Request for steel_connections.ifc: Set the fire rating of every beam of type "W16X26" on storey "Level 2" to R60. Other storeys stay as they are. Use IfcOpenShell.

First a look at what the model holds.

```python
import ifcopenshell
import ifcopenshell.util.element

model = ifcopenshell.open("steel_connections.ifc")
print(model.schema)
storey = next(s for s in model.by_type("IfcBuildingStorey") if s.Name == "Level 2")
beams = [e for e in ifcopenshell.util.element.get_decomposition(storey) if e.is_a("IfcBeam")]
seen = {}
for e in beams:
    element_type = ifcopenshell.util.element.get_type(e)
    key = (element_type.Name if element_type != e and element_type else None, ifcopenshell.util.element.get_pset(e, "Pset_BeamCommon", "FireRating"))
    seen[key] = seen.get(key, 0) + 1
for (name, value), count in sorted(seen.items(), key=str):
    print(count, "x", name, "|", value)
```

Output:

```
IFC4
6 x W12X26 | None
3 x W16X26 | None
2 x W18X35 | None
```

```python
import ifcopenshell
import ifcopenshell.api.pset
import ifcopenshell.util.element

model = ifcopenshell.open("steel_connections.ifc")

storey = next(s for s in model.by_type("IfcBuildingStorey") if s.Name == "Level 2")
beams = [e for e in ifcopenshell.util.element.get_decomposition(storey) if e.is_a("IfcBeam")]

count = 0
for e in beams:
    element_type = ifcopenshell.util.element.get_type(e)
    if element_type in (None, e) or element_type.Name != "W16X26":
        continue
    # add_pset returns the element's existing set when there is one.
    pset = ifcopenshell.api.pset.add_pset(model, product=e, name="Pset_BeamCommon")
    ifcopenshell.api.pset.edit_pset(model, pset=pset, properties={"FireRating": "R60"})
    count += 1

print(count, "beams updated")

model.write("steel_connections_v2.ifc")
```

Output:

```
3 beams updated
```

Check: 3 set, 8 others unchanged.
